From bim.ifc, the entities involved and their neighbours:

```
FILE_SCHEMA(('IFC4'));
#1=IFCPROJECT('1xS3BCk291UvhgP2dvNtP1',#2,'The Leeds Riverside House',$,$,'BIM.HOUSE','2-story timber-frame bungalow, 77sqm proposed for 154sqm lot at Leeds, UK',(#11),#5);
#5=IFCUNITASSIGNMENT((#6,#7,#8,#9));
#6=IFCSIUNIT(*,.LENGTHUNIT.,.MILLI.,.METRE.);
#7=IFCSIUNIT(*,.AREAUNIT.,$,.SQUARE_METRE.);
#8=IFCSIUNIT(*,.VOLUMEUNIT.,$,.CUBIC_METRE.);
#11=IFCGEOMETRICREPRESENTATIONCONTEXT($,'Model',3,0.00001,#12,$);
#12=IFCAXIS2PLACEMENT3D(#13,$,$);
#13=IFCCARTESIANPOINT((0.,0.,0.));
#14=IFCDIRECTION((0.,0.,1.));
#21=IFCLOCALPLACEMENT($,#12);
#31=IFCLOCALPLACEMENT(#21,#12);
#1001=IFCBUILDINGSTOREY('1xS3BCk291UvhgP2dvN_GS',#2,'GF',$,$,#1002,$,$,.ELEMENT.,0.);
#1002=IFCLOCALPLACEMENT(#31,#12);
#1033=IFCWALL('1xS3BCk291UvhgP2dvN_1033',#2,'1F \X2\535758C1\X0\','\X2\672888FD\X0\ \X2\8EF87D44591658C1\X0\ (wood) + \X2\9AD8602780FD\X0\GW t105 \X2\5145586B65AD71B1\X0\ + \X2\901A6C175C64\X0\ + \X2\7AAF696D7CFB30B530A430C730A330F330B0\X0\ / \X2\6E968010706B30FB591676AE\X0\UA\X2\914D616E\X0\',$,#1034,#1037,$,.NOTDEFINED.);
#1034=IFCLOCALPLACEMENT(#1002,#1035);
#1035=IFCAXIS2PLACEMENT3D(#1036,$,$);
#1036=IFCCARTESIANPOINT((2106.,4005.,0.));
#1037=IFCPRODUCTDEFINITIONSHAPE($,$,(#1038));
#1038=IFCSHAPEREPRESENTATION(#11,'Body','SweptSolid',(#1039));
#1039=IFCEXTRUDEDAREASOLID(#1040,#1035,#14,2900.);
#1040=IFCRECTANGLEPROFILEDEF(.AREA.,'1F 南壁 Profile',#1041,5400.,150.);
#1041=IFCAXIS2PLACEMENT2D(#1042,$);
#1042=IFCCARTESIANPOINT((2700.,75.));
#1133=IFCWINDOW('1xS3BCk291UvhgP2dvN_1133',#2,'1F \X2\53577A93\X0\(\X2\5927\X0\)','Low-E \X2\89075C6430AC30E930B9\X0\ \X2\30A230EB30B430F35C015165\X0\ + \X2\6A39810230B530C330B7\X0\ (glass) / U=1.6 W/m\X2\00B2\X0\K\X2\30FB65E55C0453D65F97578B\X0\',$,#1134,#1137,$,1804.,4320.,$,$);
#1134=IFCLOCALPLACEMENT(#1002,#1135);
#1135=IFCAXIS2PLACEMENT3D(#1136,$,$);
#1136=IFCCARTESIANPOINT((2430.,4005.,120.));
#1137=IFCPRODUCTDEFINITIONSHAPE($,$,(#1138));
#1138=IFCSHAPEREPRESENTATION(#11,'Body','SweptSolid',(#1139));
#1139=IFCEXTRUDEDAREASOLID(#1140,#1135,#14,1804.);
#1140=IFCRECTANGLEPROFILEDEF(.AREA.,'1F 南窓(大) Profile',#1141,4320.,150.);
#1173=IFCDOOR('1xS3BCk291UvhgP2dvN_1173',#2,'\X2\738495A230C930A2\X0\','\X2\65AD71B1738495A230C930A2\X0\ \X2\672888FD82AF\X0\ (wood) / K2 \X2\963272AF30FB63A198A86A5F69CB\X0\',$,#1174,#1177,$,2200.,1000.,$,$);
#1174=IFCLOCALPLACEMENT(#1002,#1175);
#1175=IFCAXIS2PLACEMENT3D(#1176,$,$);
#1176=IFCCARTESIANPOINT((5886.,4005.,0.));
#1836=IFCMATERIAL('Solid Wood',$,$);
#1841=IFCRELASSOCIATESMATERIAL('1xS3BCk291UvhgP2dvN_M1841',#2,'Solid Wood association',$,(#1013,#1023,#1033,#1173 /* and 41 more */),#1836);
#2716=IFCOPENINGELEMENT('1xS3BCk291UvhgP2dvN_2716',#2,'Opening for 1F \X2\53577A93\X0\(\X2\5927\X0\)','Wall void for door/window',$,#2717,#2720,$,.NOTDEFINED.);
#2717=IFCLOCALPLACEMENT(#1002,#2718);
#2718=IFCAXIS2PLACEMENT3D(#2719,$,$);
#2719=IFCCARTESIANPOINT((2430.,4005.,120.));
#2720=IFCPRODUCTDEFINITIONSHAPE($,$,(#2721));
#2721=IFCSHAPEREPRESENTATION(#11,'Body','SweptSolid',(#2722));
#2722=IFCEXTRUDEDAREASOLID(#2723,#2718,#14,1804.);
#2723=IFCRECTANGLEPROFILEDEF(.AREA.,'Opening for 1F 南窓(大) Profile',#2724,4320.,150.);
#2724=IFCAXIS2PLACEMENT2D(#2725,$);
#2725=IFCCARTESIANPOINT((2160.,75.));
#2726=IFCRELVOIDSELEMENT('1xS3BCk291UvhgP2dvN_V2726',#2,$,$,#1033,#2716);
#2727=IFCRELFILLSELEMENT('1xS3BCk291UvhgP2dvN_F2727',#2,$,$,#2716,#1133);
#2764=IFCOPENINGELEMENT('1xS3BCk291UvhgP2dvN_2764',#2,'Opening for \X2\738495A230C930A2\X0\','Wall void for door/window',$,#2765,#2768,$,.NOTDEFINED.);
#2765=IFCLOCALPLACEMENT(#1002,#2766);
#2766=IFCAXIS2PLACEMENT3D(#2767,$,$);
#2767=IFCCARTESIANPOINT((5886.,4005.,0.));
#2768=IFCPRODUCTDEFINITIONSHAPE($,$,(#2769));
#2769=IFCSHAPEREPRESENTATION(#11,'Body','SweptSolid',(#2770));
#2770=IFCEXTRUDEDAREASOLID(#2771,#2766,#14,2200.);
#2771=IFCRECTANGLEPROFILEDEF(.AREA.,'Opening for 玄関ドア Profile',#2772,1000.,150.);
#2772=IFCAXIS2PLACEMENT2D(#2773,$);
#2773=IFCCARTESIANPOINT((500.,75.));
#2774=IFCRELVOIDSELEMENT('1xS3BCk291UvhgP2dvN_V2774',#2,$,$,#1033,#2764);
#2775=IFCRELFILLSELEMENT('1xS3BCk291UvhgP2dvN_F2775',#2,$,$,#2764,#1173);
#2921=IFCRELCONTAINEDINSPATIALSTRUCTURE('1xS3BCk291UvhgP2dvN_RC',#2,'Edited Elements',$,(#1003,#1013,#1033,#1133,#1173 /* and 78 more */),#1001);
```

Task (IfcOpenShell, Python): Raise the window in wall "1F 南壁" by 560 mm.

```python
import numpy as np
import ifcopenshell
import ifcopenshell.api.geometry
import ifcopenshell.util.placement
import ifcopenshell.util.unit

model = ifcopenshell.open("bim.ifc")
unit_scale = ifcopenshell.util.unit.calculate_unit_scale(model)

window = model.by_guid("1xS3BCk291UvhgP2dvN_1133")
opening = window.FillsVoids[0].RelatingOpeningElement
dz = 0.56 / unit_scale

shift = np.array([0.0, 0.0, dz])
# The window is not placed relative to its opening, so move both.
for product in (opening, window):
    matrix = ifcopenshell.util.placement.get_local_placement(product.ObjectPlacement)
    matrix[:3, 3] += shift
    ifcopenshell.api.geometry.edit_object_placement(model, product=product, matrix=matrix, is_si=False)

print(f"moved by {dz * unit_scale:+.3f} m")

model.write("bim_updated.ifc")
```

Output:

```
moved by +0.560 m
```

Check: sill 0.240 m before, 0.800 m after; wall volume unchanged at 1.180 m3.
